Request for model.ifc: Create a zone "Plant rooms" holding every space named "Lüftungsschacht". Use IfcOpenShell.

First a look at what the model holds.

```python
import ifcopenshell

model = ifcopenshell.open("model.ifc")
print(model.schema)
seen = {}
for space in model.by_type("IfcSpace"):
    seen[space.LongName] = seen.get(space.LongName, 0) + 1
for name, count in sorted(seen.items(), key=str):
    print(count, "x", name)
print("zones:", [z.Name for z in model.by_type("IfcZone")][:20])
```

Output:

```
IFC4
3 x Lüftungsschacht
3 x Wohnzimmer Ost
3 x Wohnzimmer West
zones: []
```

```python
import ifcopenshell
import ifcopenshell.api.group
import ifcopenshell.api.root

model = ifcopenshell.open("model.ifc")

names = {"Lüftungsschacht"}
spaces = [s for s in model.by_type("IfcSpace") if s.LongName in names]

zone = ifcopenshell.api.root.create_entity(model, ifc_class="IfcZone", name="Plant rooms")
ifcopenshell.api.group.assign_group(model, products=spaces, group=zone)
print(len(spaces), "spaces in", zone.Name)

model.write("model_rev.ifc")
```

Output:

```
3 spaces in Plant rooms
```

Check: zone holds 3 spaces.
